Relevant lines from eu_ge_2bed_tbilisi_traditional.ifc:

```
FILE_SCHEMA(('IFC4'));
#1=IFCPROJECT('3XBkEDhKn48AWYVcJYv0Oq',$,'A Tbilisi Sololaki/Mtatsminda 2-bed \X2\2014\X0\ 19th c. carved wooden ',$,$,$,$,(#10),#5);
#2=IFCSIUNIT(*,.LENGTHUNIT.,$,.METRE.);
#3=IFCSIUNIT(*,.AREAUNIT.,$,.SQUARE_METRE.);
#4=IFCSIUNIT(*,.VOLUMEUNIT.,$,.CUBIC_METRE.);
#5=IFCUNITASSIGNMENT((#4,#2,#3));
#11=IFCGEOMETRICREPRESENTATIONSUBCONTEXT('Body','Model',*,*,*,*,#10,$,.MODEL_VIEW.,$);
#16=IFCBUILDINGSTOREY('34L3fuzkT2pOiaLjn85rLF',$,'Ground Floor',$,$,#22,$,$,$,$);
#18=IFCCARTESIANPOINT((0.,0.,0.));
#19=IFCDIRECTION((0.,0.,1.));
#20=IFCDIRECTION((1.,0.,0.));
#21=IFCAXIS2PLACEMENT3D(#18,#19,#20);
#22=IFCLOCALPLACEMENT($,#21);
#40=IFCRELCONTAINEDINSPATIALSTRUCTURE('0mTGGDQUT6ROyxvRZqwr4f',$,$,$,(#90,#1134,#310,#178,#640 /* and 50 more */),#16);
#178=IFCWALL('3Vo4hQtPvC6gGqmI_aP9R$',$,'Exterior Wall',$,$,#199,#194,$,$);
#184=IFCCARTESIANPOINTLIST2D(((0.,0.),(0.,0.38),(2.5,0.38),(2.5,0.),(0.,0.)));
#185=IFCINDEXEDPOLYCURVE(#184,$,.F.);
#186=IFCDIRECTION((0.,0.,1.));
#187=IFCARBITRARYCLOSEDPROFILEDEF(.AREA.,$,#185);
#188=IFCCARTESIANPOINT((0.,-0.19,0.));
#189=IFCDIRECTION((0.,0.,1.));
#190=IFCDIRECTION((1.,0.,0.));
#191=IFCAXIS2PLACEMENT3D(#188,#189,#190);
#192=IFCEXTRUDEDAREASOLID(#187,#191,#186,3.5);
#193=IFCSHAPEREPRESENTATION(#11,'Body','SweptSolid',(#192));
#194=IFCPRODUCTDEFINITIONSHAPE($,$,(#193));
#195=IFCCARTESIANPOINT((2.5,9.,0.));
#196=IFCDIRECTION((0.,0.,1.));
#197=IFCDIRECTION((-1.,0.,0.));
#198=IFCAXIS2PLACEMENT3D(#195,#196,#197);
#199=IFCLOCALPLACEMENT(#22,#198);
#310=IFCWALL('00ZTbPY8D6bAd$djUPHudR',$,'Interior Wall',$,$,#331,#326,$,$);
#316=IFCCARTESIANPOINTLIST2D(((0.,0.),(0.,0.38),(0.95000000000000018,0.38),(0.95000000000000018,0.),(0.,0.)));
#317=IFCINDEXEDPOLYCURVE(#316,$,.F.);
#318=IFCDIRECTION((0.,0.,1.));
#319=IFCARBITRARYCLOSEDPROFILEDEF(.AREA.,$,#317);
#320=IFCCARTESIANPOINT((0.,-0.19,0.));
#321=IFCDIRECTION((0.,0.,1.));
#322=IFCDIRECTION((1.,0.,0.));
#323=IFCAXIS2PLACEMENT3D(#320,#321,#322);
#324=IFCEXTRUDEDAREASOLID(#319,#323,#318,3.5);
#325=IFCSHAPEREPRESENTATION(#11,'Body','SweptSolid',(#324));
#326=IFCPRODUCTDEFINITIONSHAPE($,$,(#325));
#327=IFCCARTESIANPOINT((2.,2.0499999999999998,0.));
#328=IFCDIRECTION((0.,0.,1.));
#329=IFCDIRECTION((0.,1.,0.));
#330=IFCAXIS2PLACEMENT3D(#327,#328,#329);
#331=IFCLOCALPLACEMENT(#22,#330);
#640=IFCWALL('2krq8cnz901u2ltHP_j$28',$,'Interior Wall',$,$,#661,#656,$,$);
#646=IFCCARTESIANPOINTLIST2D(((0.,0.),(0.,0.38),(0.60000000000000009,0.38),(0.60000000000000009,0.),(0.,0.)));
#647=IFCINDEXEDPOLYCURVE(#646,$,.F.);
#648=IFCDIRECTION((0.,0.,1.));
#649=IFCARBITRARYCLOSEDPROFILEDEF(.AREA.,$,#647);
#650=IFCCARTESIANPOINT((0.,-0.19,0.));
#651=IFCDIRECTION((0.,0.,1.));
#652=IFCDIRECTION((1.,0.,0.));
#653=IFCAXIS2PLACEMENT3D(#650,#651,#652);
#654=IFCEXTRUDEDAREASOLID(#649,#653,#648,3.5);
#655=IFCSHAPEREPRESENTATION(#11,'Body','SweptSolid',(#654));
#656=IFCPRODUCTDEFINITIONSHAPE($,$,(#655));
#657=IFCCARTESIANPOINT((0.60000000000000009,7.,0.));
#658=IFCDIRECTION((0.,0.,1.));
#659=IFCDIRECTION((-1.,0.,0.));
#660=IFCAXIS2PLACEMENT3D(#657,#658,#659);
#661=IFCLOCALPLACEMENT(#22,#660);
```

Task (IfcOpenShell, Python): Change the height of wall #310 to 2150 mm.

```python
import ifcopenshell
import ifcopenshell.geom
import ifcopenshell.util.representation
import ifcopenshell.util.shape

model = ifcopenshell.open("eu_ge_2bed_tbilisi_traditional.ifc")
settings = ifcopenshell.geom.settings()


def volume(element):
    """Net volume in cubic metres, openings subtracted."""
    shape = ifcopenshell.geom.create_shape(settings, element)
    return ifcopenshell.util.shape.get_volume(shape.geometry)


wall = model.by_id(310)
before = volume(wall)

body = ifcopenshell.util.representation.get_representation(wall, "Model", "Body")
solid = body.Items[0]
old_height = solid.Depth
solid.Depth = 2.15
after = volume(wall)

print(f"height {old_height:g} -> {solid.Depth:g}, volume {before:.3f} -> {after:.3f} m3")

model.write("eu_ge_2bed_tbilisi_traditional_edited.ifc")
```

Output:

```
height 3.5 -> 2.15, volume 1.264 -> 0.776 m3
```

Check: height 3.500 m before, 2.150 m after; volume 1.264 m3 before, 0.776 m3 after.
